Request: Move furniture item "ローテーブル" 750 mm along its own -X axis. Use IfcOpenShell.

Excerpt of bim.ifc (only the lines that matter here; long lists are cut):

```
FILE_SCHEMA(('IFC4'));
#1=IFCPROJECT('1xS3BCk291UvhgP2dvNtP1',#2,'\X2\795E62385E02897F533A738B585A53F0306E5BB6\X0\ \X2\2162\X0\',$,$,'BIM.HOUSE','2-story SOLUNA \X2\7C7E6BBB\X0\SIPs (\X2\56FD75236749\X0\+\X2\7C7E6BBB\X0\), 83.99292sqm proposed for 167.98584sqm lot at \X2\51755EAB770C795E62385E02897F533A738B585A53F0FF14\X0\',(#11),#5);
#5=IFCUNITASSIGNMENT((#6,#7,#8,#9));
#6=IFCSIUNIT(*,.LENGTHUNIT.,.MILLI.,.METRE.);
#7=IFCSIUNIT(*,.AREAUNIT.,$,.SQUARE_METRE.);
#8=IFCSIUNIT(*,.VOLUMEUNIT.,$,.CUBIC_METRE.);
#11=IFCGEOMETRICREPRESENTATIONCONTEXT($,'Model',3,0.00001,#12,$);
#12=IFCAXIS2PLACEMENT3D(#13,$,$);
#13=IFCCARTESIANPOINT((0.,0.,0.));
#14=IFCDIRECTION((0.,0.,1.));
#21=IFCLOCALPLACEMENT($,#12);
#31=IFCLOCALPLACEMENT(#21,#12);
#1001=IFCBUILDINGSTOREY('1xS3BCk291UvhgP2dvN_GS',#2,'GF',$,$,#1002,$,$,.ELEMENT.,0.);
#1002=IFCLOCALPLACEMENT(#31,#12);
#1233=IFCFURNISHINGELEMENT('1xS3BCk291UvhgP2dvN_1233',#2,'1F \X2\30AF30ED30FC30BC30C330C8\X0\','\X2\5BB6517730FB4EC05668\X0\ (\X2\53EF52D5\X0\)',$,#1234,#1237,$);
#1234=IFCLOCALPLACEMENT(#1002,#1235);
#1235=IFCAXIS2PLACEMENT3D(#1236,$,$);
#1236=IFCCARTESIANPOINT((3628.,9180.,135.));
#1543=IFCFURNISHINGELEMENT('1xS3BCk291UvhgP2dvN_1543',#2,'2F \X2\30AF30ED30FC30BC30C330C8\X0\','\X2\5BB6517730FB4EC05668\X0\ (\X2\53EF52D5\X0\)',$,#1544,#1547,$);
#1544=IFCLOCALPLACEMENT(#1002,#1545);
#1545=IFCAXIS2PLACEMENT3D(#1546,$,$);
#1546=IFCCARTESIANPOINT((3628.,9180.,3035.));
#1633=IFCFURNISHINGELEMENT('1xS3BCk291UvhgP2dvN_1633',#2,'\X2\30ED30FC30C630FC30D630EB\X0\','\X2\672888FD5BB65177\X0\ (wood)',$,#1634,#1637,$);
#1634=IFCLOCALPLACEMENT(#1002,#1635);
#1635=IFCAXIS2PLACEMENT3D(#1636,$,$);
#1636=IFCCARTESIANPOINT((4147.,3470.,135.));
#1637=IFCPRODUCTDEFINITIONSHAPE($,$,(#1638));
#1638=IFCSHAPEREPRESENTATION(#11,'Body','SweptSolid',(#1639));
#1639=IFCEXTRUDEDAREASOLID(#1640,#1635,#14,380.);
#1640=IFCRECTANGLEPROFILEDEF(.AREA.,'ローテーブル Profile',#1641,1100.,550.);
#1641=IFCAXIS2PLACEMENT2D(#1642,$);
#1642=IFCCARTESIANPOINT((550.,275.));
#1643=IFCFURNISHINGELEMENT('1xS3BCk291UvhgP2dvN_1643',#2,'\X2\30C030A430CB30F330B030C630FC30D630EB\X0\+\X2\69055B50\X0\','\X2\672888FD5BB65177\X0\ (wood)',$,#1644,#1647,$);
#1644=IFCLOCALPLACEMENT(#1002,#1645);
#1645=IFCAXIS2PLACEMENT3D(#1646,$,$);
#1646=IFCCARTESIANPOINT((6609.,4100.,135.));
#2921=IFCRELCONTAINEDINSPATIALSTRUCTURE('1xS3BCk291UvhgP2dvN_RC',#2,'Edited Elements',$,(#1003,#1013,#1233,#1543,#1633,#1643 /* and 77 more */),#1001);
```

```python
import ifcopenshell
import ifcopenshell.api.geometry
import ifcopenshell.util.placement
import ifcopenshell.util.unit

model = ifcopenshell.open("bim.ifc")
unit_scale = ifcopenshell.util.unit.calculate_unit_scale(model)

item = model.by_guid("1xS3BCk291UvhgP2dvN_1633")
matrix = ifcopenshell.util.placement.get_local_placement(item.ObjectPlacement)
matrix[:3, 3] -= matrix[:3, 0] * 0.75 / unit_scale
ifcopenshell.api.geometry.edit_object_placement(model, product=item, matrix=matrix, is_si=False)

print(ifcopenshell.util.placement.get_local_placement(item.ObjectPlacement).round(3) + 0.0)

model.write("bim_updated.ifc")
```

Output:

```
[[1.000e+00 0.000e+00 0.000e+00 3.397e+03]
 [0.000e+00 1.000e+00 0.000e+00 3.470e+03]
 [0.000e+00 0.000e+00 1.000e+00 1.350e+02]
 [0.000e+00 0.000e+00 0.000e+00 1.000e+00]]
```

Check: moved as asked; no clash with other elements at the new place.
